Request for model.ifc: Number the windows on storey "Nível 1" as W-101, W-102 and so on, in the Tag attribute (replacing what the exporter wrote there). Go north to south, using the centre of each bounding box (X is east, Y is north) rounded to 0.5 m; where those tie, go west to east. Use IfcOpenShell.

First a look at what the model holds.

```python
import ifcopenshell
import ifcopenshell.util.element
import ifcopenshell.util.placement

model = ifcopenshell.open("model.ifc")
print(model.schema)
storey = next(s for s in model.by_type("IfcBuildingStorey") if s.Name == "Nível 1")
windows = [e for e in ifcopenshell.util.element.get_decomposition(storey) if e.is_a("IfcWindow")]
for e in sorted(windows, key=lambda e: e.id()):
    origin = ifcopenshell.util.placement.get_local_placement(e.ObjectPlacement)[:3, 3]
    print(e.id(), e.Tag, e.Name, origin.round(2) + 0.0, sep=" | ")
```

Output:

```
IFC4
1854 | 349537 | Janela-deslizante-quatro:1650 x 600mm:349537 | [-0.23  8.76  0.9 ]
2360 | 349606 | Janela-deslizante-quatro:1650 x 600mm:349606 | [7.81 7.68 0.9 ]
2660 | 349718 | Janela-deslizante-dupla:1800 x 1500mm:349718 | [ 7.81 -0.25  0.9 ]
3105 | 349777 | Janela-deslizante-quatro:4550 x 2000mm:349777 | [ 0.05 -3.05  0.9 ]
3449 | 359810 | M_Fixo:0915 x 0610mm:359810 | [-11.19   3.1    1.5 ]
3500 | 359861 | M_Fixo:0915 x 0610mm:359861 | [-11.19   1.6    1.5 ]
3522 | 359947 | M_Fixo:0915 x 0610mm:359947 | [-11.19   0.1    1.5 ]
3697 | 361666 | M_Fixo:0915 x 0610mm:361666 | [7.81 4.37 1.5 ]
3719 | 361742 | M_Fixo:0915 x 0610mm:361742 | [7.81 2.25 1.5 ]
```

```python
import ifcopenshell
import ifcopenshell.geom
import ifcopenshell.util.element
import ifcopenshell.util.shape

model = ifcopenshell.open("model.ifc")
settings = ifcopenshell.geom.settings()
settings.set("use-world-coords", True)


def centre(element):
    shape = ifcopenshell.geom.create_shape(settings, element)
    return ifcopenshell.util.shape.get_bbox_centroid(shape.geometry)


storey = next(s for s in model.by_type("IfcBuildingStorey") if s.Name == "Nível 1")
windows = [e for e in ifcopenshell.util.element.get_decomposition(storey) if e.is_a("IfcWindow")]

# Insertion points can sit at a corner or the storey origin, so sort by the geometry (in metres).
centres = {e: centre(e) for e in windows}
windows.sort(key=lambda e: (-round(centres[e][1] / 0.5), centres[e][0]))

for i, e in enumerate(windows, start=1):
    number = f"W-1{i:02d}"
    e.Tag = number
    print(e.id(), number)

model.write("model_edited.ifc")
```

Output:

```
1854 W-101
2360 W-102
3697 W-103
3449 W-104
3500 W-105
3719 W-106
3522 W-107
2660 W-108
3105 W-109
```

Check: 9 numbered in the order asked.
